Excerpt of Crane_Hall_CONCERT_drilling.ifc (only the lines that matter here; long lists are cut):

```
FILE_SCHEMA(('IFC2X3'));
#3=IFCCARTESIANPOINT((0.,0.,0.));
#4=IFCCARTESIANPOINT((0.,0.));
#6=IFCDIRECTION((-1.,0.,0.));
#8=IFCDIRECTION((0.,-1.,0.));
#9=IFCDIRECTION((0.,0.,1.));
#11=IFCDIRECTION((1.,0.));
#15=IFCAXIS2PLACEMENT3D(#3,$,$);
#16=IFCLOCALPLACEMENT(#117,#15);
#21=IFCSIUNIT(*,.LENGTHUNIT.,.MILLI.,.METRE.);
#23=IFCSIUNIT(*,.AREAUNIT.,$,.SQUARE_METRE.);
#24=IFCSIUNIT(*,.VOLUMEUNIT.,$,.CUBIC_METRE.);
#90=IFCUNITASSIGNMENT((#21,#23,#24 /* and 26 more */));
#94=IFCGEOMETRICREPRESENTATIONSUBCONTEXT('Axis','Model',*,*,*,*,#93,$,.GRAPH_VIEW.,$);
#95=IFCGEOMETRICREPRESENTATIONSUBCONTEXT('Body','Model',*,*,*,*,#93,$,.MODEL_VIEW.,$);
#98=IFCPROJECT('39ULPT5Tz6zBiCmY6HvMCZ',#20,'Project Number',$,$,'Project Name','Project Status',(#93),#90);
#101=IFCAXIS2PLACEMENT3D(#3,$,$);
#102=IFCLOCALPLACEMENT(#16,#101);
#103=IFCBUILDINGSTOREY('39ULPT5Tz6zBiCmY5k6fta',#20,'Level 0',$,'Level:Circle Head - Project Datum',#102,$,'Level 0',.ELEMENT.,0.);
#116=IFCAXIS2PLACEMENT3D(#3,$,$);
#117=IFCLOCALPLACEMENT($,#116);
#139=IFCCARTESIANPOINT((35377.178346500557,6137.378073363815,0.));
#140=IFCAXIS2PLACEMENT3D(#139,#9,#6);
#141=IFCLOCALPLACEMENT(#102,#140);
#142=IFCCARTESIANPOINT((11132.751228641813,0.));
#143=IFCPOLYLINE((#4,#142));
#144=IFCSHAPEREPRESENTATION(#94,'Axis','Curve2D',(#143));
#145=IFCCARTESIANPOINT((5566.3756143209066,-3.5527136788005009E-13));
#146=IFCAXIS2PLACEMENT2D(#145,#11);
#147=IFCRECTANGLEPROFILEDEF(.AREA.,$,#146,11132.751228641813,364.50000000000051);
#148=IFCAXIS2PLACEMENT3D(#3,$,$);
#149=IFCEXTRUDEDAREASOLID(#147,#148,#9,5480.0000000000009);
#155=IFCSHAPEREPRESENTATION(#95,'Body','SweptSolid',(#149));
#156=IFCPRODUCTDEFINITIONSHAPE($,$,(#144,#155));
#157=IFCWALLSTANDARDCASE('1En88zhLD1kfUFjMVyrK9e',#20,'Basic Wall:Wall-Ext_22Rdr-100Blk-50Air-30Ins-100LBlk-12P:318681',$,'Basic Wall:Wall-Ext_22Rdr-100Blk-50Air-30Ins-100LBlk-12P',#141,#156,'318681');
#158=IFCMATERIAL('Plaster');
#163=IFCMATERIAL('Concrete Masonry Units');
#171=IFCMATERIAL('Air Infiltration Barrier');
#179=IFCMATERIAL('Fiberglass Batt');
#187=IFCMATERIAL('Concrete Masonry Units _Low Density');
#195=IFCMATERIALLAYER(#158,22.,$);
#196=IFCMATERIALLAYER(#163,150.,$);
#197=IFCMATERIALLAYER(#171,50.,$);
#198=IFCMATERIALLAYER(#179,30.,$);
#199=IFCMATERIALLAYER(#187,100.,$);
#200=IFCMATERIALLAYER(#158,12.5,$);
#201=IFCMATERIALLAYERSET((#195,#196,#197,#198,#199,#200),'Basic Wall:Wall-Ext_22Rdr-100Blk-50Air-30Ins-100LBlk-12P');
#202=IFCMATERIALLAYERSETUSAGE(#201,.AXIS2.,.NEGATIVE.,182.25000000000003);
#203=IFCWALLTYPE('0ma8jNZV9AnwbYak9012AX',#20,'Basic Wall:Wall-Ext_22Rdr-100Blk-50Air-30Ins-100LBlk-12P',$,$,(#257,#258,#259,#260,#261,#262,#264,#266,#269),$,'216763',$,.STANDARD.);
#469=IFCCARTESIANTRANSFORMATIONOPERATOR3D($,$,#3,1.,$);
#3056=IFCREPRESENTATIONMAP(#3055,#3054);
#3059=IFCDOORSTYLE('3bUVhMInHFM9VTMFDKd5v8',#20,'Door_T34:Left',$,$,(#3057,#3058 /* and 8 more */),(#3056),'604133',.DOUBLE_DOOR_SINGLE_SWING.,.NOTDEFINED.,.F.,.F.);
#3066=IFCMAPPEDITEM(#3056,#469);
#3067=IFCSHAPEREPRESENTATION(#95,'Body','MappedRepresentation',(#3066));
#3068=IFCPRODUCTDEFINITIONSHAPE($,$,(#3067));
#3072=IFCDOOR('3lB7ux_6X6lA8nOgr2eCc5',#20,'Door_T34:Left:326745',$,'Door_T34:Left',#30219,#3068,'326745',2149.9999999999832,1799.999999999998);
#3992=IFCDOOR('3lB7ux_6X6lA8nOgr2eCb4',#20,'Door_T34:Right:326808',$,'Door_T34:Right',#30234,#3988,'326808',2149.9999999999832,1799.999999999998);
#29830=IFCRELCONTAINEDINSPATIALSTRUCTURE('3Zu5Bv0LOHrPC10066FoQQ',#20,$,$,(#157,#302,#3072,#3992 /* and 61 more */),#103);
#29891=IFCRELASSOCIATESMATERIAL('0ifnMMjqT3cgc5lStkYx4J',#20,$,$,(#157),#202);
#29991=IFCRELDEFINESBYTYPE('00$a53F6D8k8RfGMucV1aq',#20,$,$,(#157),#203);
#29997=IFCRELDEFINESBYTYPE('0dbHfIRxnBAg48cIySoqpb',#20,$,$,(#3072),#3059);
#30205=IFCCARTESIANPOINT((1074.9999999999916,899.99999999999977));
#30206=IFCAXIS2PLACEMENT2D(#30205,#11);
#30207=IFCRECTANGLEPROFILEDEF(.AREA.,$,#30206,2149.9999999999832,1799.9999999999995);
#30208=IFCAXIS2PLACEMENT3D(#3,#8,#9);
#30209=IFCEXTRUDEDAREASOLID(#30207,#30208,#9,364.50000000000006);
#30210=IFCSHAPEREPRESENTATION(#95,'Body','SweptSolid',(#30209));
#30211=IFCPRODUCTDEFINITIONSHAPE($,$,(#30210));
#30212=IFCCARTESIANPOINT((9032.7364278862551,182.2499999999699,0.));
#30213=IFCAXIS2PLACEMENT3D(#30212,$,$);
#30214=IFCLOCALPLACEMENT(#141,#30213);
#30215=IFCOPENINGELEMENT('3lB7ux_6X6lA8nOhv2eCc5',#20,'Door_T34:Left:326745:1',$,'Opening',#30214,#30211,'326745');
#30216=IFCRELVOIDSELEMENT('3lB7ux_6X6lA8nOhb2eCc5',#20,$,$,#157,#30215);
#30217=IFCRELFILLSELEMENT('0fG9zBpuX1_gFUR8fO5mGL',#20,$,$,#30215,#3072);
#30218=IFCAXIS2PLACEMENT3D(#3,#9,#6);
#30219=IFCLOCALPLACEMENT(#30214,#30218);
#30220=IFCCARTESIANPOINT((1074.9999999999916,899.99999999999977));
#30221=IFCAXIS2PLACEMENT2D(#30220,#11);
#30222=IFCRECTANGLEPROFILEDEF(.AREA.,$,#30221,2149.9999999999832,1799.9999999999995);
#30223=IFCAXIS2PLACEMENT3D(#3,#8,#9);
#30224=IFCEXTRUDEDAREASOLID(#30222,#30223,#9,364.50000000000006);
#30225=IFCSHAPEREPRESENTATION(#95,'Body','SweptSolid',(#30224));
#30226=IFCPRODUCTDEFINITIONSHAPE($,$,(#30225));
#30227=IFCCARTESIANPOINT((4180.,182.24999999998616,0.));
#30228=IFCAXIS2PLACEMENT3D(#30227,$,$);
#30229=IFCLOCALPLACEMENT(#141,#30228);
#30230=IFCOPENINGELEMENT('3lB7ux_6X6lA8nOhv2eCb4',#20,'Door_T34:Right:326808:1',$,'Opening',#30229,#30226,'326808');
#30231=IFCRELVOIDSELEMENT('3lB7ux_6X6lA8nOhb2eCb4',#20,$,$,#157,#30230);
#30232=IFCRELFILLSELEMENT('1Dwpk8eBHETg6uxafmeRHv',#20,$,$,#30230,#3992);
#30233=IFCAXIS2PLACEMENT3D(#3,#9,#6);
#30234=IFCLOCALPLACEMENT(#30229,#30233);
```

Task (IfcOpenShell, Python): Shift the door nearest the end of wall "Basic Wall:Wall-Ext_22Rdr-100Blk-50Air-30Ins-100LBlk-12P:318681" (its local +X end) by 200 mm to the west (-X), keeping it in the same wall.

```python
import ifcopenshell
import ifcopenshell.api.geometry
import ifcopenshell.util.placement
import ifcopenshell.util.unit

model = ifcopenshell.open("Crane_Hall_CONCERT_drilling.ifc")
unit_scale = ifcopenshell.util.unit.calculate_unit_scale(model)

door = model.by_guid("3lB7ux_6X6lA8nOgr2eCc5")
opening = door.FillsVoids[0].RelatingOpeningElement
wall = opening.VoidsElements[0].RelatingBuildingElement

wall_matrix = ifcopenshell.util.placement.get_local_placement(wall.ObjectPlacement)
shift = wall_matrix[:3, 0] * 0.2 / unit_scale
before = ifcopenshell.util.placement.get_local_placement(door.ObjectPlacement)[:3, 3].copy()

# The door is placed relative to its opening, so it follows when the opening moves.
matrix = ifcopenshell.util.placement.get_local_placement(opening.ObjectPlacement)
matrix[:3, 3] += shift
ifcopenshell.api.geometry.edit_object_placement(
    model, product=opening, matrix=matrix, is_si=False, should_transform_children=True
)

after = ifcopenshell.util.placement.get_local_placement(door.ObjectPlacement)[:3, 3]
print("door moved by", (after - before).round(3) + 0.0)

model.write("Crane_Hall_CONCERT_drilling-out.ifc")
```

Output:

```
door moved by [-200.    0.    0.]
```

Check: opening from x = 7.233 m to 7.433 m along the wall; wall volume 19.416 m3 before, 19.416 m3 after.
